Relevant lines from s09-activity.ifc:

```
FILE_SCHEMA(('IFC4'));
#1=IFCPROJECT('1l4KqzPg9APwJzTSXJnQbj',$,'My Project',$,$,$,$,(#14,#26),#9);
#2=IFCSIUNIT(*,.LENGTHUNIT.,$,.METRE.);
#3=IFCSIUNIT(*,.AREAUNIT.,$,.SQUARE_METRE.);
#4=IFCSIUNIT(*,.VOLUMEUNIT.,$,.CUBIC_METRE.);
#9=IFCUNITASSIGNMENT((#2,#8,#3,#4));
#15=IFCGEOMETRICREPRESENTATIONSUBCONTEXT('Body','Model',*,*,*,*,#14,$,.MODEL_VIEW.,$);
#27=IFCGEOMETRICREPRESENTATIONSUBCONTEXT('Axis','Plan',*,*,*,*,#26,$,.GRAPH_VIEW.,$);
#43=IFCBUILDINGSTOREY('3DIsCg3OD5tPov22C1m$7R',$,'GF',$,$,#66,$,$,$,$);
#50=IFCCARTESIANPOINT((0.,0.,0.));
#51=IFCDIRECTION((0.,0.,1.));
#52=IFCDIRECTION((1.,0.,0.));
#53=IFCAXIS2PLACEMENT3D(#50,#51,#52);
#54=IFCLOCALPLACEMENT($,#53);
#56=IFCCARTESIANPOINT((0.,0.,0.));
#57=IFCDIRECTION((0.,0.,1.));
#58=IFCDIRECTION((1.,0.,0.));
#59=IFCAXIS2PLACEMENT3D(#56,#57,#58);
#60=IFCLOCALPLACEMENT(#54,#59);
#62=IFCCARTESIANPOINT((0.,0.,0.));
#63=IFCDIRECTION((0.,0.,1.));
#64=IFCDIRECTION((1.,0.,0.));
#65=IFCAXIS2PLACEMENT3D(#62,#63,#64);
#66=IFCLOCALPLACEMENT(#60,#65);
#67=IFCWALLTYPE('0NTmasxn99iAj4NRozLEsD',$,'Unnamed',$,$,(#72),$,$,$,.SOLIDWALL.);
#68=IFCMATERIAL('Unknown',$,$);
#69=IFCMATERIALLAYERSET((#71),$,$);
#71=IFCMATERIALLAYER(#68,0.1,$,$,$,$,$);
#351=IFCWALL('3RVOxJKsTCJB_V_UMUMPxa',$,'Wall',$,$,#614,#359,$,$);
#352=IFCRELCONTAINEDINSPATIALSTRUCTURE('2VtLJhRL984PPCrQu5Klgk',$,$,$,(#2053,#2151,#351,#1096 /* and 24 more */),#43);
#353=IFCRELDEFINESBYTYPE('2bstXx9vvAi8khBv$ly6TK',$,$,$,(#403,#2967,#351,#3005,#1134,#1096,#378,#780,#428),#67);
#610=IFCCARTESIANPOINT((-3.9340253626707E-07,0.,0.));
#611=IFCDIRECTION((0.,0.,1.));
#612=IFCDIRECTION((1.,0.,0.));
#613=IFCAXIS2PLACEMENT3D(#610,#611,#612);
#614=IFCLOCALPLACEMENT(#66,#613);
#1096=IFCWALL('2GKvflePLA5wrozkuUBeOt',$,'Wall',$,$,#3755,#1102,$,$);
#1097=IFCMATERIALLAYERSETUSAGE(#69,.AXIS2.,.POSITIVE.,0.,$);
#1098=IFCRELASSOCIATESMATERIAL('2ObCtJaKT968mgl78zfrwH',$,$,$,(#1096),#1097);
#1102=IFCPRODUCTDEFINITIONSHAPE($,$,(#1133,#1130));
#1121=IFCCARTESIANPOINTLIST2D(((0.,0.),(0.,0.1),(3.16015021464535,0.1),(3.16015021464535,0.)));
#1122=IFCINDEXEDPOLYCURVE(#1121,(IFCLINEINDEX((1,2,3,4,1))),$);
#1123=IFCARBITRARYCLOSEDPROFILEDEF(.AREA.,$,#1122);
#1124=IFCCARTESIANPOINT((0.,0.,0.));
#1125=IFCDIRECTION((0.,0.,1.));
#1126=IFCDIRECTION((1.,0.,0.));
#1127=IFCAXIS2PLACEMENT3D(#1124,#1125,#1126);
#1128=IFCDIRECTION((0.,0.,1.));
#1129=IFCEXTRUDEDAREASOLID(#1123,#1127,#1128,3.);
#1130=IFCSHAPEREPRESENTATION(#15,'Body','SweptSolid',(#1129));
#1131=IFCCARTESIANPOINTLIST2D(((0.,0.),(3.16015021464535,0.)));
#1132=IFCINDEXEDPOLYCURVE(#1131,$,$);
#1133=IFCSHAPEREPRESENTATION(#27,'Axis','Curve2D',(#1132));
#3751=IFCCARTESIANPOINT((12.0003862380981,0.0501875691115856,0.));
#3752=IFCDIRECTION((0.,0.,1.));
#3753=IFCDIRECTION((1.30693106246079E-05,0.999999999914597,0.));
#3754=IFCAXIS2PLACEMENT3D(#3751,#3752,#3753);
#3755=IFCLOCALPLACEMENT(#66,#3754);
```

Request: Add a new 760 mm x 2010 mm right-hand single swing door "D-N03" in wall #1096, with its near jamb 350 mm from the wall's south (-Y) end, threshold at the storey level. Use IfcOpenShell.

```python
import numpy as np
import ifcopenshell
import ifcopenshell.api.feature
import ifcopenshell.api.geometry
import ifcopenshell.api.root
import ifcopenshell.api.spatial
import ifcopenshell.geom
import ifcopenshell.util.element
import ifcopenshell.util.placement
import ifcopenshell.util.representation
import ifcopenshell.util.shape
import ifcopenshell.util.unit

model = ifcopenshell.open("s09-activity.ifc")
unit_scale = ifcopenshell.util.unit.calculate_unit_scale(model)
settings = ifcopenshell.geom.settings()


def volume(element):
    """Net volume in cubic metres, openings subtracted."""
    shape = ifcopenshell.geom.create_shape(settings, element)
    return ifcopenshell.util.shape.get_volume(shape.geometry)


wall = model.by_guid("2GKvflePLA5wrozkuUBeOt")
storey = ifcopenshell.util.element.get_container(wall, ifc_class="IfcBuildingStorey")
context = ifcopenshell.util.representation.get_context(model, "Model", "Body", "MODEL_VIEW")
before = volume(wall)

width, height, from_end, sill = 0.76, 2.01, 0.35, 0.0  # metres

# The wall runs along its own X axis, and the end named is its -X end.
wall_shape = ifcopenshell.geom.create_shape(settings, wall)
x, y, z = ifcopenshell.util.shape.get_vertices(wall_shape.geometry).T
start = x.min() + from_end
face, thickness = float(y.min()), float(y.max() - y.min())
wall_matrix = ifcopenshell.util.placement.get_local_placement(wall.ObjectPlacement)
level = ifcopenshell.util.placement.get_local_placement(storey.ObjectPlacement)[2, 3]


def in_wall(x, y):
    """Placement at x, y metres in the wall's axes, at sill height."""
    matrix = wall_matrix.copy()
    matrix[:, 3] = wall_matrix @ np.array([x / unit_scale, y / unit_scale, 0.0, 1.0])
    matrix[2, 3] = level + sill / unit_scale
    return matrix


# Opening: a box that overshoots both wall faces by 50 mm.
opening = ifcopenshell.api.root.create_entity(model, ifc_class="IfcOpeningElement", predefined_type="OPENING")
box = ifcopenshell.api.geometry.add_wall_representation(
    model, context=context, length=width, height=height, thickness=thickness + 0.1
)
ifcopenshell.api.geometry.assign_representation(model, product=opening, representation=box)
ifcopenshell.api.geometry.edit_object_placement(model, product=opening, matrix=in_wall(start, face - 0.05), is_si=False)
ifcopenshell.api.feature.add_feature(model, feature=opening, element=wall)

door = ifcopenshell.api.root.create_entity(model, ifc_class="IfcDoor", name="D-N03", predefined_type="DOOR")
door.OverallWidth, door.OverallHeight = width / unit_scale, height / unit_scale
door.OperationType = "SINGLE_SWING_RIGHT"
body = ifcopenshell.api.geometry.add_door_representation(
    model,
    context=context,
    overall_width=door.OverallWidth,
    overall_height=door.OverallHeight,
    operation_type="SINGLE_SWING_RIGHT",
    lining_properties={"LiningDepth": thickness / unit_scale, "ThresholdDepth": thickness / unit_scale},
)
ifcopenshell.api.geometry.assign_representation(model, product=door, representation=body)
ifcopenshell.api.spatial.assign_container(model, products=[door], relating_structure=storey)
ifcopenshell.api.feature.add_filling(model, opening=opening, element=door)

# The lining spans the wall, so the door starts at the wall face.
ifcopenshell.api.geometry.edit_object_placement(model, product=door, matrix=in_wall(start, face), is_si=False)

after = volume(wall)

print(f"wall volume {before:.3f} -> {after:.3f} m3")

model.write("s09-activity_v2.ifc")
```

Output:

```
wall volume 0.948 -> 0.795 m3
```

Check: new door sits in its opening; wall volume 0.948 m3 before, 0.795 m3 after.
